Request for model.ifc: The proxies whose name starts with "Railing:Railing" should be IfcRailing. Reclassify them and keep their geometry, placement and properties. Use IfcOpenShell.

First a look at what the model holds.

```python
import re

import ifcopenshell

model = ifcopenshell.open("model.ifc")
print(model.schema)
seen = {}
for e in model.by_type("IfcBuildingElementProxy"):
    name = re.sub(r":\d+(:\d+)?$", "", e.Name or "")  # drop the element id that some exporters append
    seen[name] = seen.get(name, 0) + 1
for name, count in sorted(seen.items()):
    print(count, "x", name)
```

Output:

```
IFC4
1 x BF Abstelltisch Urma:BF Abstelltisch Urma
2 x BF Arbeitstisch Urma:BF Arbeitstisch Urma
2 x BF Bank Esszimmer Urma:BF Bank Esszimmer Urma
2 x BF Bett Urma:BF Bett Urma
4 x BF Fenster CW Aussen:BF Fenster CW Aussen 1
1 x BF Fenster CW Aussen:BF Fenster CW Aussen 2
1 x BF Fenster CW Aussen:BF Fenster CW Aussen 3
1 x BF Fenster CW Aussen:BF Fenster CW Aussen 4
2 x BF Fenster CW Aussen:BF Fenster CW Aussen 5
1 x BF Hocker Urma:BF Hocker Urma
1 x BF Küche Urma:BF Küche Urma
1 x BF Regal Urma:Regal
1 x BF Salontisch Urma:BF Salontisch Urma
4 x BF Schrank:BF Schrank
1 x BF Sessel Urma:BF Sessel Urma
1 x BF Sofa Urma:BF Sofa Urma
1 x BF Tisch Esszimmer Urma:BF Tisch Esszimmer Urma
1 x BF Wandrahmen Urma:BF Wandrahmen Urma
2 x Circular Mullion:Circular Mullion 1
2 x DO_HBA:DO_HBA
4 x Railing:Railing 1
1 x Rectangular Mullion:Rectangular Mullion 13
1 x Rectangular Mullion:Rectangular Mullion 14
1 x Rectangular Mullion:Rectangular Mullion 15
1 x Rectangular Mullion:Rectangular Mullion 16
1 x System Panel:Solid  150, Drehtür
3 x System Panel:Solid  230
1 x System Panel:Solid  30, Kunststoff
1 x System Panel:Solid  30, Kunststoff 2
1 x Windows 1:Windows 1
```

```python
import ifcopenshell
import ifcopenshell.api.root

model = ifcopenshell.open("model.ifc")

proxies = [e.id() for e in model.by_type("IfcBuildingElementProxy") if (e.Name or "").startswith("Railing:Railing")]
for step_id in proxies:
    proxy = model.by_id(step_id)
    ifcopenshell.api.root.reassign_class(model, product=proxy, ifc_class="IfcRailing")

print(sum(model.by_id(i).is_a("IfcRailing") for i in proxies), "reclassified")

model.write("model_rev.ifc")
```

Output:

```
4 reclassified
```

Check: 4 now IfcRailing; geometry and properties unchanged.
